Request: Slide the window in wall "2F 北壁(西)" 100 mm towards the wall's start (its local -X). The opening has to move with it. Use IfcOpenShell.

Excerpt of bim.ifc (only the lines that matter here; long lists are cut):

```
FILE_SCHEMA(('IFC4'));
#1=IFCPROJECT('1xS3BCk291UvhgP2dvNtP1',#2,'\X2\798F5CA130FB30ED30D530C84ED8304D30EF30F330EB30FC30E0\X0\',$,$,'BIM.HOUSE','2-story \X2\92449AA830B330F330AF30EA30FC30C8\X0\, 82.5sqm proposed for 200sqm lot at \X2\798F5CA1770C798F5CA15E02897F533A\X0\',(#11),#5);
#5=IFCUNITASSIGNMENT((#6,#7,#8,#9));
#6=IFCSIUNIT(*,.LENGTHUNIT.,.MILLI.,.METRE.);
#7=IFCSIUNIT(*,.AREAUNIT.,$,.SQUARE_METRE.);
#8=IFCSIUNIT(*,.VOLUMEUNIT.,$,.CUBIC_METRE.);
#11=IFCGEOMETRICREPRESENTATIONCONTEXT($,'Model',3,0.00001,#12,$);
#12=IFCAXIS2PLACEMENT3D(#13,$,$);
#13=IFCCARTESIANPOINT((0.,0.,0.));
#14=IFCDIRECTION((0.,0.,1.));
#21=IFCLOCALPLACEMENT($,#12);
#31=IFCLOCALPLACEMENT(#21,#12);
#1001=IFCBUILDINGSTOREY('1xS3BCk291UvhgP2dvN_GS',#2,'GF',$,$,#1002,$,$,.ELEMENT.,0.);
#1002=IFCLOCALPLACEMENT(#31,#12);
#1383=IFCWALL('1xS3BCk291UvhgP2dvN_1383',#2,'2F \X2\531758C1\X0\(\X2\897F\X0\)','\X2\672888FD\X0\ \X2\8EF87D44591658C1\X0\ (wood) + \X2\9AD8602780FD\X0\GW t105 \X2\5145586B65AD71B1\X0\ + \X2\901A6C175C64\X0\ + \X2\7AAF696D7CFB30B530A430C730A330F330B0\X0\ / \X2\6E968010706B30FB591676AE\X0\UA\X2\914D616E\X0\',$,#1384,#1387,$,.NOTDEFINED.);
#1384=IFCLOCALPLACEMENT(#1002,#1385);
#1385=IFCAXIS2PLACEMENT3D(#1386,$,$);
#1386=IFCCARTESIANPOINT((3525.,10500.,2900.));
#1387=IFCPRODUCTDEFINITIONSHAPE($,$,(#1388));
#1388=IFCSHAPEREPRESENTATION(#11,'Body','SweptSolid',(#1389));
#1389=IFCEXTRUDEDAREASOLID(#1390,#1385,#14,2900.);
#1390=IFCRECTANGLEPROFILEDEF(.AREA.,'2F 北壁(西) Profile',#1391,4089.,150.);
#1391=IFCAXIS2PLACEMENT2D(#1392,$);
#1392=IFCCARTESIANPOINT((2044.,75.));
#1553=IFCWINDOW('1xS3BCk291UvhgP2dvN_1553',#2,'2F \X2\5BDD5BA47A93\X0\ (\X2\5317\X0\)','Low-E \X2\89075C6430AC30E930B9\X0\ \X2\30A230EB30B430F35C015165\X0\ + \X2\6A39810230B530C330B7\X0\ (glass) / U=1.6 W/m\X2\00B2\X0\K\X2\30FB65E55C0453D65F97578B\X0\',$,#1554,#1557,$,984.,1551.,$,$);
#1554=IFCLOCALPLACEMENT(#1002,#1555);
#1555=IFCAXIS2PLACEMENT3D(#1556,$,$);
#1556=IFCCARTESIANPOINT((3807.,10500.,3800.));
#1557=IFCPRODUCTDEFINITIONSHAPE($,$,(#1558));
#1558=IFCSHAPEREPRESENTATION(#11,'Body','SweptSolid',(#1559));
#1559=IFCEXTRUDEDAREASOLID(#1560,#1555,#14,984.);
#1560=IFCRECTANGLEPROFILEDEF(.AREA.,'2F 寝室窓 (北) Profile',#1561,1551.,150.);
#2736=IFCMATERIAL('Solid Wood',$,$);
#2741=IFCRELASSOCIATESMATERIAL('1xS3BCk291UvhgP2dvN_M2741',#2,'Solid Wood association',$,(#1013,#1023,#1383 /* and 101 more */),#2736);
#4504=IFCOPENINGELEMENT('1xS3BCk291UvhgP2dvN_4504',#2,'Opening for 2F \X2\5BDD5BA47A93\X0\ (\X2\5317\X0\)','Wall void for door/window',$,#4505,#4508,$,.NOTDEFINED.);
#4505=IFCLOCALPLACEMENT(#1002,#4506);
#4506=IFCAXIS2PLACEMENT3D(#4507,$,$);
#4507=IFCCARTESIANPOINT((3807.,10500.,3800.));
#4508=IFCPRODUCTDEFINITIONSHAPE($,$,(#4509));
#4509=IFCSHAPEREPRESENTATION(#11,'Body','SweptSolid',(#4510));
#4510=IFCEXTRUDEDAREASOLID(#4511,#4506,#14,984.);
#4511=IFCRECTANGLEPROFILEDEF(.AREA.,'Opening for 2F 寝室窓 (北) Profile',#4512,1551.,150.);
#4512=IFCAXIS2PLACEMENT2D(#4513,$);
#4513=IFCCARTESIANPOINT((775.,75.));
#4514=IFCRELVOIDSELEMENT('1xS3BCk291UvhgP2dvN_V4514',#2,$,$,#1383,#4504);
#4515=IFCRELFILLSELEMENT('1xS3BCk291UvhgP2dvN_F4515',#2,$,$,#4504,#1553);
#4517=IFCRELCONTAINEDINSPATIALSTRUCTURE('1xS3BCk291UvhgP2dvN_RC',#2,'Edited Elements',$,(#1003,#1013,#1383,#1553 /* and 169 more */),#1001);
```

```python
import ifcopenshell
import ifcopenshell.api.geometry
import ifcopenshell.util.placement
import ifcopenshell.util.unit

model = ifcopenshell.open("bim.ifc")
unit_scale = ifcopenshell.util.unit.calculate_unit_scale(model)

window = model.by_guid("1xS3BCk291UvhgP2dvN_1553")
opening = window.FillsVoids[0].RelatingOpeningElement
wall = opening.VoidsElements[0].RelatingBuildingElement

wall_matrix = ifcopenshell.util.placement.get_local_placement(wall.ObjectPlacement)
shift = wall_matrix[:3, 0] * -0.1 / unit_scale
before = ifcopenshell.util.placement.get_local_placement(window.ObjectPlacement)[:3, 3].copy()

# The window is not placed relative to its opening, so move both.
for product in (opening, window):
    matrix = ifcopenshell.util.placement.get_local_placement(product.ObjectPlacement)
    matrix[:3, 3] += shift
    ifcopenshell.api.geometry.edit_object_placement(model, product=product, matrix=matrix, is_si=False)

after = ifcopenshell.util.placement.get_local_placement(window.ObjectPlacement)[:3, 3]
print("window moved by", (after - before).round(3) + 0.0)

model.write("bim_v2.ifc")
```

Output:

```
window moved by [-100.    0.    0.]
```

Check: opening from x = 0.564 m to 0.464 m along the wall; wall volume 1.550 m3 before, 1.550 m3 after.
